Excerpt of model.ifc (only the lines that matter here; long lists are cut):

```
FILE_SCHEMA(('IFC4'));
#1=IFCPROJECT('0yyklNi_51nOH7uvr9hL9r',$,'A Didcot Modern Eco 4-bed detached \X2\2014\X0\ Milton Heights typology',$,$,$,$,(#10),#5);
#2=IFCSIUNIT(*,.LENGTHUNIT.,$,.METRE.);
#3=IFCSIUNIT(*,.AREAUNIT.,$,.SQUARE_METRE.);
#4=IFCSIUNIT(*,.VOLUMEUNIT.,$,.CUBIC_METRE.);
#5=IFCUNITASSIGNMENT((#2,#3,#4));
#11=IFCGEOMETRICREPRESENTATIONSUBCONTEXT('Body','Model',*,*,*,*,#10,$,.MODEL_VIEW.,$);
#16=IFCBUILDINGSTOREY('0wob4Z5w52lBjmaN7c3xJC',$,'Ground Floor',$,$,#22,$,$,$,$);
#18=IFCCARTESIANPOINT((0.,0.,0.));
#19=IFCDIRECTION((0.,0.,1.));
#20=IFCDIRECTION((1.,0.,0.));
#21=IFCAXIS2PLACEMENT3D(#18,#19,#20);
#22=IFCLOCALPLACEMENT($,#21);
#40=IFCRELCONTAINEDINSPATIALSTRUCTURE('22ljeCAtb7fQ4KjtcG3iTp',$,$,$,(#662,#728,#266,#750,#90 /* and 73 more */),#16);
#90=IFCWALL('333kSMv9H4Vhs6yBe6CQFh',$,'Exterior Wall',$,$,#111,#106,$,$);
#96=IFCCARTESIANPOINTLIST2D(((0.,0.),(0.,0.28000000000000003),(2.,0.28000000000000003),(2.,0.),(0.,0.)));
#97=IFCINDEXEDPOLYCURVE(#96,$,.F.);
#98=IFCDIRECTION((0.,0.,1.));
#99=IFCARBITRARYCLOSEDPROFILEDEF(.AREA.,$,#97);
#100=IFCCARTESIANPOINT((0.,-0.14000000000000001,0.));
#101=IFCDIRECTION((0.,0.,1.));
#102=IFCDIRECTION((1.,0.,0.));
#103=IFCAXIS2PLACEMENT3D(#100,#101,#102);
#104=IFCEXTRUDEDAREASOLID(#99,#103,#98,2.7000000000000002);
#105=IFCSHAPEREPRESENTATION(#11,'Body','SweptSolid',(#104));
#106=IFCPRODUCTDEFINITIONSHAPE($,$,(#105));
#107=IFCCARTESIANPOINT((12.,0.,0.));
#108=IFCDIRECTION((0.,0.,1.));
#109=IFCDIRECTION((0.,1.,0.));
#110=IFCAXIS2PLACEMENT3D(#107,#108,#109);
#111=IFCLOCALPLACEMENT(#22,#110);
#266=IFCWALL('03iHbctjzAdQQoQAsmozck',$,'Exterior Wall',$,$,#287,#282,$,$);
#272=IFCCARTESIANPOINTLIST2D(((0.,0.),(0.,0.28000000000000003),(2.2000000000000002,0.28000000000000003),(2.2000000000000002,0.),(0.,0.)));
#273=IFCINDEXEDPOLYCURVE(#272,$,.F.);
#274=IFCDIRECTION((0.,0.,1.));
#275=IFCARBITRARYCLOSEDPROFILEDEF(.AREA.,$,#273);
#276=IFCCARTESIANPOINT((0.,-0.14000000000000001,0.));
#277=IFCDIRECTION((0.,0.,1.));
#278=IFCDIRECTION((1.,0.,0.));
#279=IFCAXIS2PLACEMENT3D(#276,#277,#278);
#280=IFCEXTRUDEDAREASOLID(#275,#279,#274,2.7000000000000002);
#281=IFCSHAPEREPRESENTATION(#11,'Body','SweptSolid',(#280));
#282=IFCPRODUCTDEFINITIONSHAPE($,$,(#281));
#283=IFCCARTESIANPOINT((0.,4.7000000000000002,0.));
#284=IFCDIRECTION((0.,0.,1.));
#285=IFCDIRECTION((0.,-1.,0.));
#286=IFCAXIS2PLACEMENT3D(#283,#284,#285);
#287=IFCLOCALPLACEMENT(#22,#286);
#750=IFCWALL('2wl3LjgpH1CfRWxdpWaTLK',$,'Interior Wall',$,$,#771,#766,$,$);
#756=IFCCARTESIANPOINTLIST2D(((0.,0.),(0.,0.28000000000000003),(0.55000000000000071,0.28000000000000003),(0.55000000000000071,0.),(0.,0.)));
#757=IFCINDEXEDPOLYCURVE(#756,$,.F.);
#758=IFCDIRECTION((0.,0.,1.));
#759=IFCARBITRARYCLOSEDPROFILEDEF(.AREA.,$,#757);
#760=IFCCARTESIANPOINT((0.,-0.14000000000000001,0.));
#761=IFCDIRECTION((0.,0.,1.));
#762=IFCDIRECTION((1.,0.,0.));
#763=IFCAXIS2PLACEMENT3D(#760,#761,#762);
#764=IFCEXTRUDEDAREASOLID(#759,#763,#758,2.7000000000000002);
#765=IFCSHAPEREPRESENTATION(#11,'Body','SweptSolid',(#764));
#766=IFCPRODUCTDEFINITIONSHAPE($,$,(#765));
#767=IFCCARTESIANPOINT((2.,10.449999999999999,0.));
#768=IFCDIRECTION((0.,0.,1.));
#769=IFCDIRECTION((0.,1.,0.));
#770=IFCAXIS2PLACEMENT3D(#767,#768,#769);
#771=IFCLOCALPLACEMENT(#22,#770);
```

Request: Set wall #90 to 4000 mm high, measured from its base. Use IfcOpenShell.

```python
import ifcopenshell
import ifcopenshell.geom
import ifcopenshell.util.representation
import ifcopenshell.util.shape
import ifcopenshell.util.unit

model = ifcopenshell.open("model.ifc")
unit_scale = ifcopenshell.util.unit.calculate_unit_scale(model)
settings = ifcopenshell.geom.settings()


def volume(element):
    """Net volume in cubic metres, openings subtracted."""
    shape = ifcopenshell.geom.create_shape(settings, element)
    return ifcopenshell.util.shape.get_volume(shape.geometry)


wall = model.by_id(90)
before = volume(wall)

body = ifcopenshell.util.representation.get_representation(wall, "Model", "Body")
solid = body.Items[0]
old_height = solid.Depth
solid.Depth = 4 / unit_scale
after = volume(wall)

print(f"height {old_height:g} -> {solid.Depth:g}, volume {before:.3f} -> {after:.3f} m3")

model.write("model_v2.ifc")
```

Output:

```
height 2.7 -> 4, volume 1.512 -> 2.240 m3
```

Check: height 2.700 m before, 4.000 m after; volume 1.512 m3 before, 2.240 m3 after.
